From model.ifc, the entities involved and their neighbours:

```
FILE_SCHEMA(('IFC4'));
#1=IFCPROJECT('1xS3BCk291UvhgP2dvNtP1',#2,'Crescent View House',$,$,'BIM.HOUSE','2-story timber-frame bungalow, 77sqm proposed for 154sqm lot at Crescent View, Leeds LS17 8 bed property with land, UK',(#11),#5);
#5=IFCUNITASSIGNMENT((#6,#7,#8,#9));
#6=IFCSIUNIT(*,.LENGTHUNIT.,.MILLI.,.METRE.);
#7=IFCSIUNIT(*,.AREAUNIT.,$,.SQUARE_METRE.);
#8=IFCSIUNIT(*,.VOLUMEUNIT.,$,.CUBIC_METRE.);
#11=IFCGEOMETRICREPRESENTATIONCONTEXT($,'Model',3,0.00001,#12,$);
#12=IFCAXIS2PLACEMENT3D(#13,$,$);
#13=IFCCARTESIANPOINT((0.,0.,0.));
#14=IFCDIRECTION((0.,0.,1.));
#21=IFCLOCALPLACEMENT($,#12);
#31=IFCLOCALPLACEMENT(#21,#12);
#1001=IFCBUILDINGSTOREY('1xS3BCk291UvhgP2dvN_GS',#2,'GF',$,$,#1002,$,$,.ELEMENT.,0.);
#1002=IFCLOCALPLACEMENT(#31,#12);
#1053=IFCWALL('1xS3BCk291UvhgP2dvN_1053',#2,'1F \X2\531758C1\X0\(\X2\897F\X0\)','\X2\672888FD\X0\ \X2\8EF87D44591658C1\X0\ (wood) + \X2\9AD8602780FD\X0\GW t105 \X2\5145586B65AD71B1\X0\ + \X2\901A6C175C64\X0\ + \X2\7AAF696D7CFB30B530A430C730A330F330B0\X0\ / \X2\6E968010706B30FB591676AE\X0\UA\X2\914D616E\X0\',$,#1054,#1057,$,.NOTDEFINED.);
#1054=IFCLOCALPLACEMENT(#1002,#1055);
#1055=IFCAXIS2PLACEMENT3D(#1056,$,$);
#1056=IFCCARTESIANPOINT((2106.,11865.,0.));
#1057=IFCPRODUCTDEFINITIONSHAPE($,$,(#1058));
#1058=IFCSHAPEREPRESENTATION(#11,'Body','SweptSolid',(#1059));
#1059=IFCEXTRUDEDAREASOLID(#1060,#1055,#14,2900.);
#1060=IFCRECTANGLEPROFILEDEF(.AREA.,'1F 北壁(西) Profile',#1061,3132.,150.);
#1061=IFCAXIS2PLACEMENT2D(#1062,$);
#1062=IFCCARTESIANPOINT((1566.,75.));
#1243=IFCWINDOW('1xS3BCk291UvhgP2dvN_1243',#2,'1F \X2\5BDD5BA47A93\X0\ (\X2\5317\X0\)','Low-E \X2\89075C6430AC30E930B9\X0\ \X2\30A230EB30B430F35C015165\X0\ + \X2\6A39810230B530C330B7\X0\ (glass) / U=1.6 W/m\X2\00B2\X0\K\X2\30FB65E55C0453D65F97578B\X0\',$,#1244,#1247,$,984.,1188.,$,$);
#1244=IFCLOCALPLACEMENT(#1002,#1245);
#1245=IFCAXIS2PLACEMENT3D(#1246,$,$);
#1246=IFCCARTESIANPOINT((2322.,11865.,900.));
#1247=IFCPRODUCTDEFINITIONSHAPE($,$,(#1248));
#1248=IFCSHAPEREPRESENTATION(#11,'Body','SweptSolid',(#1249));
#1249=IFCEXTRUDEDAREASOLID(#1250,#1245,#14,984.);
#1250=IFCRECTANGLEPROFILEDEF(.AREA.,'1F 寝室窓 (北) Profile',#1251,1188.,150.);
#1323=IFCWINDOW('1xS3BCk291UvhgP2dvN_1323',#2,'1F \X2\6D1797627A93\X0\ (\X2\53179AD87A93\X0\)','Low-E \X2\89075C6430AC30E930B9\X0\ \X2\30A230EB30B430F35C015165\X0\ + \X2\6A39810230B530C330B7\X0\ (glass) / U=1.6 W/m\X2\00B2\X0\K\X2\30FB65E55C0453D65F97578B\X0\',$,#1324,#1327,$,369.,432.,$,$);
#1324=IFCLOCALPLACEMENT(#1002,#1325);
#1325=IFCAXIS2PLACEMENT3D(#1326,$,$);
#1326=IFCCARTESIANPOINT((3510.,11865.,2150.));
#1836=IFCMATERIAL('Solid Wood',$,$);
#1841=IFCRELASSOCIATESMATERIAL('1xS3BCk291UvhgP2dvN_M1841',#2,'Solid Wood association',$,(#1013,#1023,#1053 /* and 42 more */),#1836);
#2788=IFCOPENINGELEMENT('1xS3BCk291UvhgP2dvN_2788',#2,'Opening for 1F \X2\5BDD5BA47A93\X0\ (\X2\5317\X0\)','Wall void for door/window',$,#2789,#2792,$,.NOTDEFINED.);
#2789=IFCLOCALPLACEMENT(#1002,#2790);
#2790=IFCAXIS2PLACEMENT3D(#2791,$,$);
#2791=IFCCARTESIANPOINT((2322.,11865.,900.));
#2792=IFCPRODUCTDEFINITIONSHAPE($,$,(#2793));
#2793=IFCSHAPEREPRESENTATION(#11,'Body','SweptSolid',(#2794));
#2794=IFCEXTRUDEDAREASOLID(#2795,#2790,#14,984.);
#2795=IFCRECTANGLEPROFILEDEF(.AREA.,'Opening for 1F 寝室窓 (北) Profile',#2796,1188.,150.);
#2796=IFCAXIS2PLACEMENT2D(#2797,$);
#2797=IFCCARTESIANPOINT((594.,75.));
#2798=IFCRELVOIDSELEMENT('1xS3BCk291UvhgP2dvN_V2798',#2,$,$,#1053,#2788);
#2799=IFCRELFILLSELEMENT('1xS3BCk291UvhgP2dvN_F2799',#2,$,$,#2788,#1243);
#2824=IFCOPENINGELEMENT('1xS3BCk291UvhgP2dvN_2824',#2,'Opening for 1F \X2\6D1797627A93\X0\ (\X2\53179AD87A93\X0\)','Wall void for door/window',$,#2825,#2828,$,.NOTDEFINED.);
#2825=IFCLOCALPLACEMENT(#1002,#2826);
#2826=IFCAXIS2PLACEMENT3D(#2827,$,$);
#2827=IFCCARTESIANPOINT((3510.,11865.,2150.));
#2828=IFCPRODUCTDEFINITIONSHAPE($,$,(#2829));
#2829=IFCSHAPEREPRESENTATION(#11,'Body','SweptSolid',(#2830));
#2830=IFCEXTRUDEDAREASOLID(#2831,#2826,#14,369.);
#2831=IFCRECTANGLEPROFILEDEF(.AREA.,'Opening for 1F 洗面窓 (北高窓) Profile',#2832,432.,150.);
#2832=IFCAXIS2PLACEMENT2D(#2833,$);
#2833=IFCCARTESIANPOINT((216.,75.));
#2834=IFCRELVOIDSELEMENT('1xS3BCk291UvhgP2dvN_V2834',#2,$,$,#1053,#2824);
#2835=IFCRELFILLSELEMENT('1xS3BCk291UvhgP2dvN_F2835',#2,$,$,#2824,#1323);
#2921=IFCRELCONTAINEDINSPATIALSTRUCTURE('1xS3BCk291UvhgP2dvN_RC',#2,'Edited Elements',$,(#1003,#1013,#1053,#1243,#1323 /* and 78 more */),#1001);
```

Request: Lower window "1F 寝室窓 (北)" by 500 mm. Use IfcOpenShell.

```python
import numpy as np
import ifcopenshell
import ifcopenshell.api.geometry
import ifcopenshell.util.placement
import ifcopenshell.util.unit

model = ifcopenshell.open("model.ifc")
unit_scale = ifcopenshell.util.unit.calculate_unit_scale(model)

window = model.by_id(1243)
opening = window.FillsVoids[0].RelatingOpeningElement
dz = -0.5 / unit_scale

shift = np.array([0.0, 0.0, dz])
# The window is not placed relative to its opening, so move both.
for product in (opening, window):
    matrix = ifcopenshell.util.placement.get_local_placement(product.ObjectPlacement)
    matrix[:3, 3] += shift
    ifcopenshell.api.geometry.edit_object_placement(model, product=product, matrix=matrix, is_si=False)

print(f"moved by {dz * unit_scale:+.3f} m")

model.write("model_v2.ifc")
```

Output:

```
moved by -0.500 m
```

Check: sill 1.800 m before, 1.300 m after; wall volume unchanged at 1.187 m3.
